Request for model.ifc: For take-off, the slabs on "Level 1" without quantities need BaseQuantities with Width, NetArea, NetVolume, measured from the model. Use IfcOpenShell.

First a look at what the model holds.

```python
import ifcopenshell
import ifcopenshell.util.element
import ifcopenshell.util.unit

model = ifcopenshell.open("model.ifc")
print(model.schema)
for unit_type in ("LENGTHUNIT", "AREAUNIT", "VOLUMEUNIT"):
    print(unit_type, ifcopenshell.util.unit.calculate_unit_scale(model, unit_type))
storey = next(s for s in model.by_type("IfcBuildingStorey") if s.Name == "Level 1")
slabs = [e for e in ifcopenshell.util.element.get_decomposition(storey) if e.is_a("IfcSlab")]
for e in sorted(slabs, key=lambda e: e.id()):
    print(e.id(), e.is_a(), e.Name, list(ifcopenshell.util.element.get_psets(e, qtos_only=True)), sep=" | ")
```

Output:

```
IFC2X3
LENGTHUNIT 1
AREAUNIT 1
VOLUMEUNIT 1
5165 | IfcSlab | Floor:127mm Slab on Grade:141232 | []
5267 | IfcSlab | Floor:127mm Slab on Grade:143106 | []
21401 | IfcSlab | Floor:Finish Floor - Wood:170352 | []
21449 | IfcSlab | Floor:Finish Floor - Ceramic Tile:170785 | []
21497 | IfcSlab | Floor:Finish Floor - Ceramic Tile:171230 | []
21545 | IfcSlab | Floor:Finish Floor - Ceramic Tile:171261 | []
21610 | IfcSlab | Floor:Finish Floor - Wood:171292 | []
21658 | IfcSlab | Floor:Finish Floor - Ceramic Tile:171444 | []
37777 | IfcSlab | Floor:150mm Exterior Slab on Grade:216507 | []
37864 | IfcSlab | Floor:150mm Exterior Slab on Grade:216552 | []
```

```python
import ifcopenshell
import ifcopenshell.api.pset
import ifcopenshell.geom
import ifcopenshell.util.element
import ifcopenshell.util.shape
import ifcopenshell.util.unit

model = ifcopenshell.open("model.ifc")
unit_scale = ifcopenshell.util.unit.calculate_unit_scale(model)
area_scale = ifcopenshell.util.unit.calculate_unit_scale(model, "AREAUNIT")
volume_scale = ifcopenshell.util.unit.calculate_unit_scale(model, "VOLUMEUNIT")
settings = ifcopenshell.geom.settings()

storey = next(s for s in model.by_type("IfcBuildingStorey") if s.Name == "Level 1")
slabs = [e for e in ifcopenshell.util.element.get_decomposition(storey) if e.is_a("IfcSlab")]

for e in sorted(slabs, key=lambda e: e.id()):
    if ifcopenshell.util.element.get_psets(e, qtos_only=True, should_inherit=False):
        continue
    # Geometry comes back in metres, in the element's own axes.
    shape = ifcopenshell.geom.create_shape(settings, e)
    values = {
        "Width": ifcopenshell.util.shape.get_z(shape.geometry) / unit_scale,
        "NetArea": ifcopenshell.util.shape.get_footprint_area(shape.geometry) / area_scale,
        "NetVolume": ifcopenshell.util.shape.get_volume(shape.geometry) / volume_scale,
    }
    qto = ifcopenshell.api.pset.add_qto(model, product=e, name="BaseQuantities")
    ifcopenshell.api.pset.edit_qto(model, qto=qto, properties=values)
    print(e.id(), {k: round(v, 3) for k, v in values.items()})

model.write("model_edited.ifc")
```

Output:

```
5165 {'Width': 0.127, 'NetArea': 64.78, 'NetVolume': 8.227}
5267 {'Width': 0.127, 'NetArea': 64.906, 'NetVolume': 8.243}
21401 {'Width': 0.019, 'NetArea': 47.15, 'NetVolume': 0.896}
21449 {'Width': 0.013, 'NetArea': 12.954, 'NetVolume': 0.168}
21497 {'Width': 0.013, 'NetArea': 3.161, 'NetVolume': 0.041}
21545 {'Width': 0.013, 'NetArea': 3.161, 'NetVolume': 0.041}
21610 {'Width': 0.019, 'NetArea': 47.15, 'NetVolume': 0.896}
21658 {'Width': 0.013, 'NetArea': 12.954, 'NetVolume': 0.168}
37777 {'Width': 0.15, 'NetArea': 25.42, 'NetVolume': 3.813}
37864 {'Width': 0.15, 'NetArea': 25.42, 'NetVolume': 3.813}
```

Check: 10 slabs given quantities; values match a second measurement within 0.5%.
